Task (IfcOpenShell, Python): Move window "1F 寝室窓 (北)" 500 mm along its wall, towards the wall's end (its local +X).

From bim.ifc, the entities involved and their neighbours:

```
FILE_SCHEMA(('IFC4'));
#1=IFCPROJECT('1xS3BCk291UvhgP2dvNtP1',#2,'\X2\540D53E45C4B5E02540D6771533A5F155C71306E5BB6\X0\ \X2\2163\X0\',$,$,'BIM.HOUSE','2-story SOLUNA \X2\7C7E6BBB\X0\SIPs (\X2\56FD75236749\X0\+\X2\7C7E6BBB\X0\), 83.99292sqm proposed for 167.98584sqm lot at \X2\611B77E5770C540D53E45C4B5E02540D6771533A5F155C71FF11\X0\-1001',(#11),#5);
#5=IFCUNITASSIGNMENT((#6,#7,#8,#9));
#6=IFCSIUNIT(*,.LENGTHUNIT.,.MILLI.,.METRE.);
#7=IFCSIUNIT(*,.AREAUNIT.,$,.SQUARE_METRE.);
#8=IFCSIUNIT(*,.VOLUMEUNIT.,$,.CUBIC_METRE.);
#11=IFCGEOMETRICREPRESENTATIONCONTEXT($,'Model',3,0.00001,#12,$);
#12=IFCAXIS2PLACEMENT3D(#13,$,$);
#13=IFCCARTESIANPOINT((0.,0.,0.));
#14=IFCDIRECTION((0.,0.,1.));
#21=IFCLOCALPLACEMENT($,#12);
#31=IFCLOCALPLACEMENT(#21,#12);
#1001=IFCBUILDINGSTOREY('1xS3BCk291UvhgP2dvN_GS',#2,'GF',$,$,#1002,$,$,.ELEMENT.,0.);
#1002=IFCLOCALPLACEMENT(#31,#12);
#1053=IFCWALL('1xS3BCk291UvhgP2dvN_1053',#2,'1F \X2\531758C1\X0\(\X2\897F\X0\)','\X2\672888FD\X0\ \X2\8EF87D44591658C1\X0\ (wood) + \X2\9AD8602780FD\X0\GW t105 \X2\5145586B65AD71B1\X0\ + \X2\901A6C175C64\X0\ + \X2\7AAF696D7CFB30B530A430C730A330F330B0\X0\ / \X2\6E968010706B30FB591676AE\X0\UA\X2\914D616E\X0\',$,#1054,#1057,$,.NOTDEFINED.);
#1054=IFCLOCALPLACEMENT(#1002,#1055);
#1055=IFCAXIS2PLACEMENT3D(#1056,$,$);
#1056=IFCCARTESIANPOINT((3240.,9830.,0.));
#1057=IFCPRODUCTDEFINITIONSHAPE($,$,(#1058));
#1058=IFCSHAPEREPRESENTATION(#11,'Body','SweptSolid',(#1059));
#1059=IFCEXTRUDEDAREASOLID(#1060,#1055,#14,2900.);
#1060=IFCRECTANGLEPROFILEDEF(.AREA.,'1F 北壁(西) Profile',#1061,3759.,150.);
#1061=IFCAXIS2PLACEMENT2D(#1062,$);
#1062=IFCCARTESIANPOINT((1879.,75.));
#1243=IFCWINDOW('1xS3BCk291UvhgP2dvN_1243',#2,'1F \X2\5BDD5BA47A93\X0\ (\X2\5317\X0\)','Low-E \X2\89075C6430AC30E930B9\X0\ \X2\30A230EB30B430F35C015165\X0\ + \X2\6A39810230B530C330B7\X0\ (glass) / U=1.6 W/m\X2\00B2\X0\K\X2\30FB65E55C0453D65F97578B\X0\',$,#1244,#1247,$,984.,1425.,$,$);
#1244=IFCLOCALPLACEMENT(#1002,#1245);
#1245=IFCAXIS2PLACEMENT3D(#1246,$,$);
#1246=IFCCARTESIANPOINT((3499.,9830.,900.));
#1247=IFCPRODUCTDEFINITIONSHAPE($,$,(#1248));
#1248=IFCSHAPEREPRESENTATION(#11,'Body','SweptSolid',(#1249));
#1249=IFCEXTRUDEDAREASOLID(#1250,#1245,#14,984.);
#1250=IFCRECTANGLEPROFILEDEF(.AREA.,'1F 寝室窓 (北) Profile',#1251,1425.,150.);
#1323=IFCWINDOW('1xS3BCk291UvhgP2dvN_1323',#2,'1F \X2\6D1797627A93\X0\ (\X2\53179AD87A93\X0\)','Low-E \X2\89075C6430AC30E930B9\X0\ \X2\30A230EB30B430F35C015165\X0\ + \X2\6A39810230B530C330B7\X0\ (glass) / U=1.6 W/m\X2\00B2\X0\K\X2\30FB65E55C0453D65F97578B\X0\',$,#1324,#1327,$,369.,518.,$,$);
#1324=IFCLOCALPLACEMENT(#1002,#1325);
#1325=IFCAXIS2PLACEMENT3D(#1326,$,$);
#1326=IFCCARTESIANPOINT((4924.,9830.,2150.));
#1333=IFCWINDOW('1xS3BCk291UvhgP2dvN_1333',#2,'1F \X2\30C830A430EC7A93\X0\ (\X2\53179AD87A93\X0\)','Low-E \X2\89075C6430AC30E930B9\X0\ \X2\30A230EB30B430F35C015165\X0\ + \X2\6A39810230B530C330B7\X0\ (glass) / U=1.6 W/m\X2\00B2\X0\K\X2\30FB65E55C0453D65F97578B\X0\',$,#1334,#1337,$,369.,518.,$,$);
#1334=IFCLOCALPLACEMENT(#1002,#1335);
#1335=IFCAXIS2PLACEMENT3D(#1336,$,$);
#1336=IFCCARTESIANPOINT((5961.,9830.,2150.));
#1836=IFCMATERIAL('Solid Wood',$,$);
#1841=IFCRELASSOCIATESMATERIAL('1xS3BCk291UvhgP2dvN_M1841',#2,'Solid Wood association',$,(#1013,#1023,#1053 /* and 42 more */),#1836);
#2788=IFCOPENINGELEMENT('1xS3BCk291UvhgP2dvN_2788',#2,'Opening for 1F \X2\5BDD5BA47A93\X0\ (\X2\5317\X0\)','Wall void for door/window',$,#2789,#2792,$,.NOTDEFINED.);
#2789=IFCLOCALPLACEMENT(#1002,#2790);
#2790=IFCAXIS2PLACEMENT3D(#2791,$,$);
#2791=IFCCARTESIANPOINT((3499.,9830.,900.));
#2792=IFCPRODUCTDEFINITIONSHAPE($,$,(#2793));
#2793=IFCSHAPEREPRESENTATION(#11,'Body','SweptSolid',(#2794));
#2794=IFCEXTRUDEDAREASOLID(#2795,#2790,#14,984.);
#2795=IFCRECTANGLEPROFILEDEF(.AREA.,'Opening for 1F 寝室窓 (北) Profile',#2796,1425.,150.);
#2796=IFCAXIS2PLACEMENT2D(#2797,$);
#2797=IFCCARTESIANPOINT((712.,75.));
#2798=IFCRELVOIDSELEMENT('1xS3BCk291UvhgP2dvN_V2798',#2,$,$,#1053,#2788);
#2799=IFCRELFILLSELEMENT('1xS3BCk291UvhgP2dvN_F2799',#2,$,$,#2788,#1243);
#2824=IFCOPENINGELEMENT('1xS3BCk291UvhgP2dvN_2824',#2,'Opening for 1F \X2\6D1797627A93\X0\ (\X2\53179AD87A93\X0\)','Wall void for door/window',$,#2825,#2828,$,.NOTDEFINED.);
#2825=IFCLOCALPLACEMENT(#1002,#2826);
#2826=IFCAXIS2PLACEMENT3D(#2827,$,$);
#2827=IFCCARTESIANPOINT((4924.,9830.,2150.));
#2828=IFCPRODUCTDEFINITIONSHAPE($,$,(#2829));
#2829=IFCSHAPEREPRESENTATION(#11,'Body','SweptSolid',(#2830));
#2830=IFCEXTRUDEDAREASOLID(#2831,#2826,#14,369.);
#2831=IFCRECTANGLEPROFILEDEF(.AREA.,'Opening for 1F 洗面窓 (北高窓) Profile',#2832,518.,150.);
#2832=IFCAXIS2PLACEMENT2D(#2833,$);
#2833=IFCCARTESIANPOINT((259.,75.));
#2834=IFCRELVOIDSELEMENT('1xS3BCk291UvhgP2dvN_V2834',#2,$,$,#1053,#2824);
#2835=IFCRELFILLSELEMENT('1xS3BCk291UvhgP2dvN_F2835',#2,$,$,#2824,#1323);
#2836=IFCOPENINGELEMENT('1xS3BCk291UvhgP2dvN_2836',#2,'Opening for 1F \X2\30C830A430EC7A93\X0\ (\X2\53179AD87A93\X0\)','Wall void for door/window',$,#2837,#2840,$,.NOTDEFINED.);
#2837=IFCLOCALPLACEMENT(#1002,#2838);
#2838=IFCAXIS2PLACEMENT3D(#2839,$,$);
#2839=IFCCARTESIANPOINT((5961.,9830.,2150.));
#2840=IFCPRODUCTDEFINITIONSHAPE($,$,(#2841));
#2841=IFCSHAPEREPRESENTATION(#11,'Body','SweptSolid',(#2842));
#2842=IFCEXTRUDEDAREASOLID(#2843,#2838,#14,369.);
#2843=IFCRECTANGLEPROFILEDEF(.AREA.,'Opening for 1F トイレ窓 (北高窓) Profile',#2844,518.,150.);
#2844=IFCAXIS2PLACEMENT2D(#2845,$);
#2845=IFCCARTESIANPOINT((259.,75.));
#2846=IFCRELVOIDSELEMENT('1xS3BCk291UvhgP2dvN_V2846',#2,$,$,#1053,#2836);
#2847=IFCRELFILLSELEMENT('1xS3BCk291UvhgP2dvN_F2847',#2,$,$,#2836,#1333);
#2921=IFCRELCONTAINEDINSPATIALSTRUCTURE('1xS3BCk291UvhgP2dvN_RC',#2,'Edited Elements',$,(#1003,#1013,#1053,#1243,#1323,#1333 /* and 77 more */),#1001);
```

```python
import ifcopenshell
import ifcopenshell.api.geometry
import ifcopenshell.util.placement
import ifcopenshell.util.unit

model = ifcopenshell.open("bim.ifc")
unit_scale = ifcopenshell.util.unit.calculate_unit_scale(model)

window = model.by_guid("1xS3BCk291UvhgP2dvN_1243")
opening = window.FillsVoids[0].RelatingOpeningElement
wall = opening.VoidsElements[0].RelatingBuildingElement

wall_matrix = ifcopenshell.util.placement.get_local_placement(wall.ObjectPlacement)
shift = wall_matrix[:3, 0] * 0.5 / unit_scale
before = ifcopenshell.util.placement.get_local_placement(window.ObjectPlacement)[:3, 3].copy()

# The window is not placed relative to its opening, so move both.
for product in (opening, window):
    matrix = ifcopenshell.util.placement.get_local_placement(product.ObjectPlacement)
    matrix[:3, 3] += shift
    ifcopenshell.api.geometry.edit_object_placement(model, product=product, matrix=matrix, is_si=False)

after = ifcopenshell.util.placement.get_local_placement(window.ObjectPlacement)[:3, 3]
print("window moved by", (after - before).round(3) + 0.0)

model.write("bim_v2.ifc")
```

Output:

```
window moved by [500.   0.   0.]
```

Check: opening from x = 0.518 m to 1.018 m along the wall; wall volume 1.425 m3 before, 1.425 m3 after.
